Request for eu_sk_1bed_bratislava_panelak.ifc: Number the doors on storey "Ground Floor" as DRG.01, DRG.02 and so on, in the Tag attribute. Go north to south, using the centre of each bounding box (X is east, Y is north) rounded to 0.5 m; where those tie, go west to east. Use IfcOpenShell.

First a look at what the model holds.

```python
import ifcopenshell
import ifcopenshell.util.element
import ifcopenshell.util.placement

model = ifcopenshell.open("eu_sk_1bed_bratislava_panelak.ifc")
print(model.schema)
storey = next(s for s in model.by_type("IfcBuildingStorey") if s.Name == "Ground Floor")
doors = [e for e in ifcopenshell.util.element.get_decomposition(storey) if e.is_a("IfcDoor")]
for e in sorted(doors, key=lambda e: e.id()):
    origin = ifcopenshell.util.placement.get_local_placement(e.ObjectPlacement)[:3, 3]
    print(e.id(), e.Tag, e.Name, origin.round(2) + 0.0, sep=" | ")
```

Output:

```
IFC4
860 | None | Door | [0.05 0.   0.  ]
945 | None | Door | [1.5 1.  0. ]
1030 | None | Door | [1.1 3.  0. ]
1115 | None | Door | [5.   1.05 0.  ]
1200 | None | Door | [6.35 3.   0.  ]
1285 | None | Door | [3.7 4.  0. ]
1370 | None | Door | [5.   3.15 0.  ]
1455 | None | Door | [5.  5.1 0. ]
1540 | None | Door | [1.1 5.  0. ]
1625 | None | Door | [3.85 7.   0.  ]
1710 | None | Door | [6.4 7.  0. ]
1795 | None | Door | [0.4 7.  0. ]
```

```python
import ifcopenshell
import ifcopenshell.geom
import ifcopenshell.util.element
import ifcopenshell.util.shape

model = ifcopenshell.open("eu_sk_1bed_bratislava_panelak.ifc")
settings = ifcopenshell.geom.settings()
settings.set("use-world-coords", True)


def centre(element):
    shape = ifcopenshell.geom.create_shape(settings, element)
    return ifcopenshell.util.shape.get_bbox_centroid(shape.geometry)


storey = next(s for s in model.by_type("IfcBuildingStorey") if s.Name == "Ground Floor")
doors = [e for e in ifcopenshell.util.element.get_decomposition(storey) if e.is_a("IfcDoor")]

# Insertion points can sit at a corner or the storey origin, so sort by the geometry (in metres).
centres = {e: centre(e) for e in doors}
doors.sort(key=lambda e: (-round(centres[e][1] / 0.5), centres[e][0]))

for i, e in enumerate(doors, start=1):
    number = f"DRG.{i:02d}"
    e.Tag = number
    print(e.id(), number)

model.write("eu_sk_1bed_bratislava_panelak_updated.ifc")
```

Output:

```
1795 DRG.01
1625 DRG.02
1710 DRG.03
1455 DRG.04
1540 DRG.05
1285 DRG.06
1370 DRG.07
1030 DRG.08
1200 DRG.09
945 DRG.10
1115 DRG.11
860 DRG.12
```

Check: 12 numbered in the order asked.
